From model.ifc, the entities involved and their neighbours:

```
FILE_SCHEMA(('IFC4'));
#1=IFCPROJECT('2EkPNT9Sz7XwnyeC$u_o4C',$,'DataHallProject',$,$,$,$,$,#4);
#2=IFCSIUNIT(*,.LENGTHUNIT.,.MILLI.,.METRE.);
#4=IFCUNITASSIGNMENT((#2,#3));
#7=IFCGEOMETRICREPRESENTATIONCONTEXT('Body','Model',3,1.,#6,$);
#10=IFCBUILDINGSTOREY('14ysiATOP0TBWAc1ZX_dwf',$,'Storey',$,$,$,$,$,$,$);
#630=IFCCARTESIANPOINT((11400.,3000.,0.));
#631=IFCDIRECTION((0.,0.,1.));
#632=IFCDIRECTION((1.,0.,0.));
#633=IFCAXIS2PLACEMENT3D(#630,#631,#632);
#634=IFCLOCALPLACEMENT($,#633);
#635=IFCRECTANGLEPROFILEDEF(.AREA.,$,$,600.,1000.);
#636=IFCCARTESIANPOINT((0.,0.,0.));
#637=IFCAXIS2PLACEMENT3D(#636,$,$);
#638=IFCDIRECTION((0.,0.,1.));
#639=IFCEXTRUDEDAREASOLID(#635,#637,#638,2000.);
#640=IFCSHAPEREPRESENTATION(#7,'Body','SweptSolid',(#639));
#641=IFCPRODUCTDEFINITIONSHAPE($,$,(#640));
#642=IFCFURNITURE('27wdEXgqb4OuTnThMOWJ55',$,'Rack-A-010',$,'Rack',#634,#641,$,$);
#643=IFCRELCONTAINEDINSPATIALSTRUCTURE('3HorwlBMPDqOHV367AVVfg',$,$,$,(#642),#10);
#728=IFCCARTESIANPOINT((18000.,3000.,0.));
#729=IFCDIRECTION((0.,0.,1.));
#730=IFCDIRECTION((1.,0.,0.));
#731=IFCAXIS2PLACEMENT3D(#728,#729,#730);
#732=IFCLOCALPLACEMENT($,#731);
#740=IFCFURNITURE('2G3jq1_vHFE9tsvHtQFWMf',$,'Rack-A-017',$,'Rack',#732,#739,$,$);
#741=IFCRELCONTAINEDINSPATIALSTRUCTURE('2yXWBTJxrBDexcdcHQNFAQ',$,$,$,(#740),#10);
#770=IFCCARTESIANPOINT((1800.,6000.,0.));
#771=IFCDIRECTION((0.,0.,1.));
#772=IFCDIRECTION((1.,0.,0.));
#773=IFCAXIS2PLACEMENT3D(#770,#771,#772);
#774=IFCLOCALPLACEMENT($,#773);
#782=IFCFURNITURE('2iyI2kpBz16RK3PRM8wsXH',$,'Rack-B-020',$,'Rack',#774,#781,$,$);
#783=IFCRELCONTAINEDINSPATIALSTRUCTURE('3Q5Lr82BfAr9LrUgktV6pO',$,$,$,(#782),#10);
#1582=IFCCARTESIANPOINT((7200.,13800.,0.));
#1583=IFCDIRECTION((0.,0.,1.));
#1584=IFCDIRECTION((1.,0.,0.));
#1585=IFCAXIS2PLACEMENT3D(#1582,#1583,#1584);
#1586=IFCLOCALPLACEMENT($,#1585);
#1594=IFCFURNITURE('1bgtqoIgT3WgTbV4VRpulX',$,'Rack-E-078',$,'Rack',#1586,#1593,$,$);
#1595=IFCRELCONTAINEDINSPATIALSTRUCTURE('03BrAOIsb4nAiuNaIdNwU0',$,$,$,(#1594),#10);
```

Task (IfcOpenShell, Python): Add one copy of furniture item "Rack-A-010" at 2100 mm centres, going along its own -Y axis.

```python
import ifcopenshell
import ifcopenshell.api.geometry
import ifcopenshell.api.root
import ifcopenshell.util.element
import ifcopenshell.util.placement
import ifcopenshell.util.unit

model = ifcopenshell.open("model.ifc")
unit_scale = ifcopenshell.util.unit.calculate_unit_scale(model)

source = model.by_guid("27wdEXgqb4OuTnThMOWJ55")
base = ifcopenshell.util.placement.get_local_placement(source.ObjectPlacement)
step = -base[:3, 1] * 2.1 / unit_scale

for i in range(1, 2):
    copy = ifcopenshell.api.root.copy_class(model, product=source)
    copy.Representation = ifcopenshell.util.element.copy_deep(
        model, source.Representation, exclude=["IfcGeometricRepresentationContext", "IfcRepresentationMap"]
    )
    matrix = base.copy()
    matrix[:3, 3] += i * step
    print("added at", matrix[:3, 3].round(3) + 0.0)
    ifcopenshell.api.geometry.edit_object_placement(model, product=copy, matrix=matrix, is_si=False)

model.write("model_edited.ifc")
```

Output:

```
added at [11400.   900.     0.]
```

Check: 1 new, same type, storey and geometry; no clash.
